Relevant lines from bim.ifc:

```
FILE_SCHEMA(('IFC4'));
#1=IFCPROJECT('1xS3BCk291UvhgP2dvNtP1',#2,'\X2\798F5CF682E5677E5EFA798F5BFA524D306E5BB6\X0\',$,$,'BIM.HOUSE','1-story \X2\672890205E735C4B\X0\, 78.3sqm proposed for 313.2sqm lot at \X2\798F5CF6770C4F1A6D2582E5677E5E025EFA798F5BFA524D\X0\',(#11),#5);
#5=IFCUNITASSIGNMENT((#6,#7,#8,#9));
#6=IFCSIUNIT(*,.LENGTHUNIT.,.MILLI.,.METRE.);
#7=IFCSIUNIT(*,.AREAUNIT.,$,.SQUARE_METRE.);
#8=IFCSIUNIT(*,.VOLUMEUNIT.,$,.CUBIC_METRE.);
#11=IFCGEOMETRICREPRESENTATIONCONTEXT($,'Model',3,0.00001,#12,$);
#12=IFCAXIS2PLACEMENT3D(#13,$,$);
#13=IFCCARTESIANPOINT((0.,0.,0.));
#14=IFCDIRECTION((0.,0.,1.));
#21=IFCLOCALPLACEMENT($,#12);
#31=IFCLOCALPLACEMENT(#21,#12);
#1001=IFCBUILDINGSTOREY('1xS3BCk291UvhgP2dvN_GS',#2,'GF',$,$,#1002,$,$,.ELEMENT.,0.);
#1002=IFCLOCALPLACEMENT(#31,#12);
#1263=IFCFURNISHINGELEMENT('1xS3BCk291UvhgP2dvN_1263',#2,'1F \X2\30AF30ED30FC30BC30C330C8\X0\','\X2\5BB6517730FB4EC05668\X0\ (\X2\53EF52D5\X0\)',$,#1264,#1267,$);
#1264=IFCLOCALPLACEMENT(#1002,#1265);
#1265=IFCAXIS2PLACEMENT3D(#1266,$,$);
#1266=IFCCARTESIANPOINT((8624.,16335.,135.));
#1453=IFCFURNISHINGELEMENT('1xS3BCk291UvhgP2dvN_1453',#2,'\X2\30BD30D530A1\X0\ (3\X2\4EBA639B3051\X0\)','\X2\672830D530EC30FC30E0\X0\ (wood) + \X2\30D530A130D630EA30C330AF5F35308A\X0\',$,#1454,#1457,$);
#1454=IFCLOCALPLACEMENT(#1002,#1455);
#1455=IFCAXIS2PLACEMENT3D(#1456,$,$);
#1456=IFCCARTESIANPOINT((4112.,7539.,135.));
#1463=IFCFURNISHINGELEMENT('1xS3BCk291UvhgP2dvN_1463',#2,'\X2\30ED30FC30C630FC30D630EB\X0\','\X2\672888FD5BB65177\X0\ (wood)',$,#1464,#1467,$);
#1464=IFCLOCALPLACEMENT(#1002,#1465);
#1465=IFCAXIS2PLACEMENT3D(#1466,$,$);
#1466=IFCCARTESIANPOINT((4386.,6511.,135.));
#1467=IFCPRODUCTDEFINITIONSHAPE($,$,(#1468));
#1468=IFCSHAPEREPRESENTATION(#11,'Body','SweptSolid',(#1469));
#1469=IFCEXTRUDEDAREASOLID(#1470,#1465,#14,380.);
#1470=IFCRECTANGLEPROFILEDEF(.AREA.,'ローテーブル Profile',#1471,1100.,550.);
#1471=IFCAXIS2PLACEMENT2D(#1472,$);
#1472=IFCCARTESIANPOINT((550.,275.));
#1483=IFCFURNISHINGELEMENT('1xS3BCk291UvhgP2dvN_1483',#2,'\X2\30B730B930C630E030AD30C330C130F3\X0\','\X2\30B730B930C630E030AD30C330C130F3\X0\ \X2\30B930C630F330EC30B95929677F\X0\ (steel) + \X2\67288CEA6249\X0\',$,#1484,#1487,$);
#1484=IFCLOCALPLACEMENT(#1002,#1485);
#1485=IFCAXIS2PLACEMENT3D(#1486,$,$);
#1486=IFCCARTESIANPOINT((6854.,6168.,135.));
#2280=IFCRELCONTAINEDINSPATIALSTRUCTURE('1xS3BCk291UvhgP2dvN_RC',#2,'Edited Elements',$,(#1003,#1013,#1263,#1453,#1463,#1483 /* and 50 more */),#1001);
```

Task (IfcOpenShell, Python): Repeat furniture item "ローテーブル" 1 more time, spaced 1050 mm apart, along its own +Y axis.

```python
import ifcopenshell
import ifcopenshell.api.geometry
import ifcopenshell.api.root
import ifcopenshell.util.element
import ifcopenshell.util.placement

model = ifcopenshell.open("bim.ifc")


def reuse_history(source, copy):
    """copy_class also copies each property set's owner history, people and application; keep the originals."""
    for rel in copy.IsDefinedBy:
        if rel.is_a("IfcRelDefinesByProperties") and (history := rel.RelatingPropertyDefinition.OwnerHistory):
            rel.RelatingPropertyDefinition.OwnerHistory = source.OwnerHistory
            ifcopenshell.util.element.remove_deep2(model, history)


source = model.by_guid("1xS3BCk291UvhgP2dvN_1463")
base = ifcopenshell.util.placement.get_local_placement(source.ObjectPlacement)
step = base[:3, 1] * 1050.0

for i in range(1, 2):
    copy = ifcopenshell.api.root.copy_class(model, product=source)
    copy.Representation = ifcopenshell.util.element.copy_deep(
        model, source.Representation, exclude=["IfcGeometricRepresentationContext", "IfcRepresentationMap"]
    )
    reuse_history(source, copy)
    matrix = base.copy()
    matrix[:3, 3] += i * step
    print("added at", matrix[:3, 3].round(3) + 0.0)
    ifcopenshell.api.geometry.edit_object_placement(model, product=copy, matrix=matrix, is_si=False)

model.write("bim-out.ifc")
```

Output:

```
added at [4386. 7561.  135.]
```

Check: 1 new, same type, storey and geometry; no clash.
